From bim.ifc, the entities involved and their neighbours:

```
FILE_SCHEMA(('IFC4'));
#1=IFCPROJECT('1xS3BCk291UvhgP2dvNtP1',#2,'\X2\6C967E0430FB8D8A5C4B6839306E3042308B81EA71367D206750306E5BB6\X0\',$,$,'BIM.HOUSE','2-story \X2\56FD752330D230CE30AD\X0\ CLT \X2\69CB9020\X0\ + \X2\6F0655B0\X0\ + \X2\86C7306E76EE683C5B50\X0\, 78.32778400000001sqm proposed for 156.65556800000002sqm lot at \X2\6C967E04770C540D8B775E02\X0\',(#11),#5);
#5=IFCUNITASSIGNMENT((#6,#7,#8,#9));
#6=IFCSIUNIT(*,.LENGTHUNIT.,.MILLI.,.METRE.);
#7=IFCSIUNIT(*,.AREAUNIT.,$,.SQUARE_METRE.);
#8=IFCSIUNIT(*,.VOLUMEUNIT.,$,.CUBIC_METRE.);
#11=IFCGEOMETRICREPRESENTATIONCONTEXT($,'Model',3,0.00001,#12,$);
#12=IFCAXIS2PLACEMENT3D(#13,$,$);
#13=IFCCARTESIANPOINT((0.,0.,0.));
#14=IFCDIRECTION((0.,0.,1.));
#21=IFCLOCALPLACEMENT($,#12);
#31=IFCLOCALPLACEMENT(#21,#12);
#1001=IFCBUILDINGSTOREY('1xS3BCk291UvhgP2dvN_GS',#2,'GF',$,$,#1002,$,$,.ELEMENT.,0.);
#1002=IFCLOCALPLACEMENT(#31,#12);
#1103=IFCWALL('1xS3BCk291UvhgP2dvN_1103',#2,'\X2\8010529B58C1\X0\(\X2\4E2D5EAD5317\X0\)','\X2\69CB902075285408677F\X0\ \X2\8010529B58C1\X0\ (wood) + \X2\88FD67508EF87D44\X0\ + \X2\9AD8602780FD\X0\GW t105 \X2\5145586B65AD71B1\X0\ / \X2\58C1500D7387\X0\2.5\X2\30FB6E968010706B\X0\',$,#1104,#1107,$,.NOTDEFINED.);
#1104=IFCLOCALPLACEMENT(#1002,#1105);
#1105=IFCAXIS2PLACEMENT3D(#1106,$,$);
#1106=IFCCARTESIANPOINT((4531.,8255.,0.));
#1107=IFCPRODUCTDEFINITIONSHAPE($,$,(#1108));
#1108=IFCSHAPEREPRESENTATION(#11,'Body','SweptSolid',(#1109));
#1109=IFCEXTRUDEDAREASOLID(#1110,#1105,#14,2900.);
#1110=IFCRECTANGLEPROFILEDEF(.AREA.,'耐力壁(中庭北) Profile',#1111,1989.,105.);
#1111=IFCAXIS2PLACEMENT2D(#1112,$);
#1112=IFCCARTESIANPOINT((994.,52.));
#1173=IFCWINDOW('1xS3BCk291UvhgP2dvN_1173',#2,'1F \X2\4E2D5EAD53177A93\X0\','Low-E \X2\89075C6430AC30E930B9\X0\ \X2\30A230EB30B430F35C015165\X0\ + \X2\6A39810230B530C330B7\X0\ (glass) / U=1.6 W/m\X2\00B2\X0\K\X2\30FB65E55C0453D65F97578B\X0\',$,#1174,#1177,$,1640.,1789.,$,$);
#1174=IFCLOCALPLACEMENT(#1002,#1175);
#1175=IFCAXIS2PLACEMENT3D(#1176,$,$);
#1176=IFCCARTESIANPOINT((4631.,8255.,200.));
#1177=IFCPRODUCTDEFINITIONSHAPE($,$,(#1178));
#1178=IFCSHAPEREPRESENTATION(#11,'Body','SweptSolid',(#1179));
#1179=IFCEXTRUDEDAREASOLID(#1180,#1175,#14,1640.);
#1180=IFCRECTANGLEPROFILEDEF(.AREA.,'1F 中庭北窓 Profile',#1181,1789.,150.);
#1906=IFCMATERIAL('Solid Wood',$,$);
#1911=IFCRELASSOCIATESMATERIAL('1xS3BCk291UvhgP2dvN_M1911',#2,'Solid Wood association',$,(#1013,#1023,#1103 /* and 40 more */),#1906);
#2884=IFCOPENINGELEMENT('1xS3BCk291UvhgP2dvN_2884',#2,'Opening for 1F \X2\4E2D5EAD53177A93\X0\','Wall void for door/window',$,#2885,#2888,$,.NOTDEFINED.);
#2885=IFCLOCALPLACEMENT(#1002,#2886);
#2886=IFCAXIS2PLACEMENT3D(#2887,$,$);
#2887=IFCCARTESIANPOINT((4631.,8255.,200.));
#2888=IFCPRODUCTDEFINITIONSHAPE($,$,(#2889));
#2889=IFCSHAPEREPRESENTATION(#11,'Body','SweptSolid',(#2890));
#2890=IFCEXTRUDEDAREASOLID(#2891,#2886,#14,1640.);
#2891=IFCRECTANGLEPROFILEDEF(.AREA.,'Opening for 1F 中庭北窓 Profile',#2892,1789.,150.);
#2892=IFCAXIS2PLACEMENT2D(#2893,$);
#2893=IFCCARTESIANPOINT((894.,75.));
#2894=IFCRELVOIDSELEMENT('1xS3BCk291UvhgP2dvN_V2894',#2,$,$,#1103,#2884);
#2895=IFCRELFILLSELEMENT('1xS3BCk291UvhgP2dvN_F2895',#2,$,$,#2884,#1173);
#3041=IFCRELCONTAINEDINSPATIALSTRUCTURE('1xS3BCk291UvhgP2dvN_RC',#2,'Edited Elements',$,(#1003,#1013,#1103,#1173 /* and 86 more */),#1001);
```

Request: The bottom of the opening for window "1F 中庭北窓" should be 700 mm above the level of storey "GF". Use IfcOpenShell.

```python
import numpy as np
import ifcopenshell
import ifcopenshell.api.geometry
import ifcopenshell.geom
import ifcopenshell.util.element
import ifcopenshell.util.placement
import ifcopenshell.util.shape
import ifcopenshell.util.unit

model = ifcopenshell.open("bim.ifc")
unit_scale = ifcopenshell.util.unit.calculate_unit_scale(model)

window = model.by_guid("1xS3BCk291UvhgP2dvN_1173")
opening = window.FillsVoids[0].RelatingOpeningElement
storey = ifcopenshell.util.element.get_container(window, ifc_class="IfcBuildingStorey")
level = ifcopenshell.util.placement.get_local_placement(storey.ObjectPlacement)[2, 3]

# The opening's origin need not be at the sill, so measure its lowest point.
shape = ifcopenshell.geom.create_shape(ifcopenshell.geom.settings(), opening)
bottom = ifcopenshell.util.shape.get_shape_bottom_elevation(shape, shape.geometry) / unit_scale
dz = level + 0.7 / unit_scale - bottom

shift = np.array([0.0, 0.0, dz])
# The window is not placed relative to its opening, so move both.
for product in (opening, window):
    matrix = ifcopenshell.util.placement.get_local_placement(product.ObjectPlacement)
    matrix[:3, 3] += shift
    ifcopenshell.api.geometry.edit_object_placement(model, product=product, matrix=matrix, is_si=False)

print(f"moved by {dz * unit_scale:+.3f} m")

model.write("bim-out.ifc")
```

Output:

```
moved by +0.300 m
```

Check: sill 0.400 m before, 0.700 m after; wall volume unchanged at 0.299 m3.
